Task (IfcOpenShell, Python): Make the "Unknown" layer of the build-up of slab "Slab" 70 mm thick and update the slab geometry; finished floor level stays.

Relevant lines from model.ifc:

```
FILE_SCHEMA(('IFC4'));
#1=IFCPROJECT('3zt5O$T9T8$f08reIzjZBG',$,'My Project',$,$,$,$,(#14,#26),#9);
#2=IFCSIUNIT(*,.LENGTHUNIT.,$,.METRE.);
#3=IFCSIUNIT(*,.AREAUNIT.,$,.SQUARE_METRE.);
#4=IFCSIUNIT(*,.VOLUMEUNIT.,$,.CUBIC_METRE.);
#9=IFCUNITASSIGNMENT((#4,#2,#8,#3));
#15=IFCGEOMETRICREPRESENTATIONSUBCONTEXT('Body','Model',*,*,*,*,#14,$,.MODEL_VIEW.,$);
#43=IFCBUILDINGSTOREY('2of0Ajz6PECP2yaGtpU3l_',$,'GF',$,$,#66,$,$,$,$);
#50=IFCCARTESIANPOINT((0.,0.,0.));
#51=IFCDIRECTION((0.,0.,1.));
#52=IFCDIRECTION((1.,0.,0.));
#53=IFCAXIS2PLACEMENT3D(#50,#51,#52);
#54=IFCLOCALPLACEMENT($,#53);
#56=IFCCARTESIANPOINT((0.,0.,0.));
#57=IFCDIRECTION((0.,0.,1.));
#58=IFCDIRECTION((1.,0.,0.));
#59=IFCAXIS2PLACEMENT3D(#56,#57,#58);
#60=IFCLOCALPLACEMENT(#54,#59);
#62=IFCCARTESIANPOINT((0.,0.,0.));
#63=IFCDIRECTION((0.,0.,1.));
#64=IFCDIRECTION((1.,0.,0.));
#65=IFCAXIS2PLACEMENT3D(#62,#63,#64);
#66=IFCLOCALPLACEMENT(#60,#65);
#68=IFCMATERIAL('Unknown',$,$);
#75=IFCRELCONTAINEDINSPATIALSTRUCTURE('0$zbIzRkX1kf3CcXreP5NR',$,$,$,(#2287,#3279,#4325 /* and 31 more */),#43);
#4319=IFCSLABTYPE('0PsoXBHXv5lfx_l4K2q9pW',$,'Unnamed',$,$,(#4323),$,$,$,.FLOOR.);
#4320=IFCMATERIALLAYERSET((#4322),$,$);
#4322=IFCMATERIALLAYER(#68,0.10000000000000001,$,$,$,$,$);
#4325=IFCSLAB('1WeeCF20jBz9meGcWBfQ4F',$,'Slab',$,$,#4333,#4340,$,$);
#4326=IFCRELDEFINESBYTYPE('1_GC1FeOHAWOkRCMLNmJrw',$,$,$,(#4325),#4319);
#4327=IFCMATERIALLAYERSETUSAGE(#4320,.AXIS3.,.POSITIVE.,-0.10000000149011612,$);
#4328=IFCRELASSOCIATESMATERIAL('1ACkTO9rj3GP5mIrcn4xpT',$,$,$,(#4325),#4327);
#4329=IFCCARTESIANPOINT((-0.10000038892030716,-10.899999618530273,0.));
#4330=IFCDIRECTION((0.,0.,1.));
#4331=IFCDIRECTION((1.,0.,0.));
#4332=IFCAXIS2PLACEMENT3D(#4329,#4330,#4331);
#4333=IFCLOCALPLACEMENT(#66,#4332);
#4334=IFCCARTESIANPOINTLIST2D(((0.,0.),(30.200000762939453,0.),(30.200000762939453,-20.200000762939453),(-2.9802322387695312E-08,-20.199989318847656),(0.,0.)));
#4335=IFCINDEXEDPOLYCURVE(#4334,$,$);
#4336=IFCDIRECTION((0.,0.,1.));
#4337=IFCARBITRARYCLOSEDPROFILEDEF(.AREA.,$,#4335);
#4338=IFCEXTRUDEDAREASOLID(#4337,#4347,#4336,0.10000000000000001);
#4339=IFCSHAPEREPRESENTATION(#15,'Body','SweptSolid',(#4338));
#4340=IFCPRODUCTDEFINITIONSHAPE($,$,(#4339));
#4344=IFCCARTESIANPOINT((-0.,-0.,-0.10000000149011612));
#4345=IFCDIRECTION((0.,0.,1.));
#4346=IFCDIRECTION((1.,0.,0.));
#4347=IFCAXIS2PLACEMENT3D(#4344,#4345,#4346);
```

```python
import ifcopenshell
import ifcopenshell.util.element
import ifcopenshell.util.representation
import ifcopenshell.util.unit

model = ifcopenshell.open("model.ifc")
unit_scale = ifcopenshell.util.unit.calculate_unit_scale(model)

layer_set = model.by_id(4320)
layer = next(l for l in layer_set.MaterialLayers if l.Material and l.Material.Name == "Unknown")
change = 0.07 / unit_scale - layer.LayerThickness
layer.LayerThickness += change

# Geometry does not follow the layer set by itself.
slabs = [e for e in ifcopenshell.util.element.get_elements_by_material(model, layer_set) if e.is_a("IfcSlab")]
for slab in sorted(slabs, key=lambda e: e.id()):
    body = ifcopenshell.util.representation.get_representation(slab, "Model", "Body")
    solid = body.Items[0]
    old_depth = solid.Depth
    solid.Depth += change
    # Extruded upwards: lower the start of the extrusion so the top stays.
    x, y, z = solid.Position.Location.Coordinates
    solid.Position.Location = model.createIfcCartesianPoint((x, y, z - change))
    print(slab.id(), f"{old_depth:g} -> {solid.Depth:g}")

# The layers are counted up from the underside, which has moved.
for usage in {ifcopenshell.util.element.get_material(slab) for slab in slabs}:
    usage.OffsetFromReferenceLine -= change

model.write("model_edited.ifc")
```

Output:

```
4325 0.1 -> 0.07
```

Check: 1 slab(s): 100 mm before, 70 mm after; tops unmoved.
